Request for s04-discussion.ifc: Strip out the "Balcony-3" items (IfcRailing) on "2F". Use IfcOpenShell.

First a look at what the model holds.

```python
import ifcopenshell
import ifcopenshell.util.element

model = ifcopenshell.open("s04-discussion.ifc")
print(model.schema)
storey = next(s for s in model.by_type("IfcBuildingStorey") if s.Name == "2F")
railings = [e for e in ifcopenshell.util.element.get_decomposition(storey) if e.is_a("IfcRailing")]
seen = {}
for e in railings:
    element_type = ifcopenshell.util.element.get_type(e)
    name = element_type.Name if element_type not in (None, e) else None
    seen[name] = seen.get(name, 0) + 1
for name, count in sorted(seen.items(), key=str):
    print(count, "x", name)
```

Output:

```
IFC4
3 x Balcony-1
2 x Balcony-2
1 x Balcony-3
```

```python
import ifcopenshell
import ifcopenshell.api.root
import ifcopenshell.util.element

model = ifcopenshell.open("s04-discussion.ifc")

storey = next(s for s in model.by_type("IfcBuildingStorey") if s.Name == "2F")
railings = [e for e in ifcopenshell.util.element.get_decomposition(storey) if e.is_a("IfcRailing")]
targets = [e for e in railings if (t := ifcopenshell.util.element.get_type(e)) not in (None, e) and t.Name == "Balcony-3"]

for e in targets:
    ifcopenshell.api.root.remove_product(model, product=e)
print(len(targets), "removed")

model.write("s04-discussion_edited.ifc")
```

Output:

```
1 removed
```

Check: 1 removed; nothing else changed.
